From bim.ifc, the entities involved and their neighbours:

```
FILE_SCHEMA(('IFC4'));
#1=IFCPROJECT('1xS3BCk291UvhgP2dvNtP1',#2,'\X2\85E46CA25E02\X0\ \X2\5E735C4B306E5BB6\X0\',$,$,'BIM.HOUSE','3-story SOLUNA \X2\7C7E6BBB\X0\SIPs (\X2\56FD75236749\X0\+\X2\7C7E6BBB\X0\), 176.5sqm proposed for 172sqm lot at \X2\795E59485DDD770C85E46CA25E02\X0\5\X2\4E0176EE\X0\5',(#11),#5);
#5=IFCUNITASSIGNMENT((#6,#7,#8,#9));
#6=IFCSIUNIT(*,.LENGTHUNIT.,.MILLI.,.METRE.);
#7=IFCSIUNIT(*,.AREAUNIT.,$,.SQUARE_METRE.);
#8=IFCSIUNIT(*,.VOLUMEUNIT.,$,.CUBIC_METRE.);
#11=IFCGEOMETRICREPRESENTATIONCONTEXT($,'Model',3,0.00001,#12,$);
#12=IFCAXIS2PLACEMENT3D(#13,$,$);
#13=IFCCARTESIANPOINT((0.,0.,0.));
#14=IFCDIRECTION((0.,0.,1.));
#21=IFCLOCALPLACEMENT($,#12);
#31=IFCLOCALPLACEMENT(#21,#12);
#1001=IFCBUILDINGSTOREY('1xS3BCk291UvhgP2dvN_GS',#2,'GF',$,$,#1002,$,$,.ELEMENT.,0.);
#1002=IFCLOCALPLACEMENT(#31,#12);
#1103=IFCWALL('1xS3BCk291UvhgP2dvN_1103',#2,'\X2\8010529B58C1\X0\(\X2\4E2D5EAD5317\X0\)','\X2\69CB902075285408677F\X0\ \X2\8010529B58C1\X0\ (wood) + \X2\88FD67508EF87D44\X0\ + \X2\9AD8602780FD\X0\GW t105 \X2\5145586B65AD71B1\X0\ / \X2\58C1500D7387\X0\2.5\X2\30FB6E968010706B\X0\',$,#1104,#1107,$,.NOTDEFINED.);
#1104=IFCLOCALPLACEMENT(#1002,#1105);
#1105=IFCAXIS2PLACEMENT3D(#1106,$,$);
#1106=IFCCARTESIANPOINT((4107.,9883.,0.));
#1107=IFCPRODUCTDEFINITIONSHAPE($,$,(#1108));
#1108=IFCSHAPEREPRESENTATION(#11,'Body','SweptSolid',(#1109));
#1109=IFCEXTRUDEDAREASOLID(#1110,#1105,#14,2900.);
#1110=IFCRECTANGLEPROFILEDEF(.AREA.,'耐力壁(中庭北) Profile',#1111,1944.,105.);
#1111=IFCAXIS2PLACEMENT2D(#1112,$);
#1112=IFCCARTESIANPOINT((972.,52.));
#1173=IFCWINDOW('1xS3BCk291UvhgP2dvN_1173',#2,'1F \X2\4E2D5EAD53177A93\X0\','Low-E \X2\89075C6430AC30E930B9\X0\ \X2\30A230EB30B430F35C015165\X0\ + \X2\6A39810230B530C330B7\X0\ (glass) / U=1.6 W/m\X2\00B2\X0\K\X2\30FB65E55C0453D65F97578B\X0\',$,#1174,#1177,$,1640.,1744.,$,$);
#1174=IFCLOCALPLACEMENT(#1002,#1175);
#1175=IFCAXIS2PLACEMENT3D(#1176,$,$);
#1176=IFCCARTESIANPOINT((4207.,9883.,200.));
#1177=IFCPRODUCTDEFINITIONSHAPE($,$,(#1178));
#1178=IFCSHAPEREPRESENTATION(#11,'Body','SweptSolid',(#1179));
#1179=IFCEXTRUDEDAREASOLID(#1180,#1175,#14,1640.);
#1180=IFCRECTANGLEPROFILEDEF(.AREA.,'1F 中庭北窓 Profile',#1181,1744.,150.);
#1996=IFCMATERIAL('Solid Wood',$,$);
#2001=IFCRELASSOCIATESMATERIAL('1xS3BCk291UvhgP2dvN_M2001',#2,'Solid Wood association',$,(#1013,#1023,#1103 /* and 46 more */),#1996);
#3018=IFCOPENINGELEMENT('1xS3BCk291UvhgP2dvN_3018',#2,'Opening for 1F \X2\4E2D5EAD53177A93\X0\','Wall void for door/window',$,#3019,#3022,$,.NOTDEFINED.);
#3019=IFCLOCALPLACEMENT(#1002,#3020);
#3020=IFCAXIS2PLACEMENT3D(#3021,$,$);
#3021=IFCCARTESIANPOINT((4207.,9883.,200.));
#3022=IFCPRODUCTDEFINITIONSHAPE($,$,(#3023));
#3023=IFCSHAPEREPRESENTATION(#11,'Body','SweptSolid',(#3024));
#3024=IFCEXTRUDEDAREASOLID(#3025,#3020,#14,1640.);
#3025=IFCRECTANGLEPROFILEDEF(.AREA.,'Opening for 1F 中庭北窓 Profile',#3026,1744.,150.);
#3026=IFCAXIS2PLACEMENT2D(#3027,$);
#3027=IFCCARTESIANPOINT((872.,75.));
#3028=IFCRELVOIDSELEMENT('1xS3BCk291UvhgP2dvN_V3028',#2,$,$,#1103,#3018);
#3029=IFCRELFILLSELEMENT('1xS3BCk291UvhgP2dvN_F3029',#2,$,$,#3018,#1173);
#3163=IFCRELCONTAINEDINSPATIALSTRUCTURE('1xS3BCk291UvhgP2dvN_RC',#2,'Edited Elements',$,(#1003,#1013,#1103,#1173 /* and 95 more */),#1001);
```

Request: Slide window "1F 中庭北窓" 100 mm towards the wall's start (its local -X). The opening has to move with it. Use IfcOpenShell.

```python
import ifcopenshell
import ifcopenshell.api.geometry
import ifcopenshell.util.placement
import ifcopenshell.util.unit

model = ifcopenshell.open("bim.ifc")
unit_scale = ifcopenshell.util.unit.calculate_unit_scale(model)

window = model.by_id(1173)
opening = window.FillsVoids[0].RelatingOpeningElement
wall = opening.VoidsElements[0].RelatingBuildingElement

wall_matrix = ifcopenshell.util.placement.get_local_placement(wall.ObjectPlacement)
shift = wall_matrix[:3, 0] * -0.1 / unit_scale
before = ifcopenshell.util.placement.get_local_placement(window.ObjectPlacement)[:3, 3].copy()

# The window is not placed relative to its opening, so move both.
for product in (opening, window):
    matrix = ifcopenshell.util.placement.get_local_placement(product.ObjectPlacement)
    matrix[:3, 3] += shift
    ifcopenshell.api.geometry.edit_object_placement(model, product=product, matrix=matrix, is_si=False)

after = ifcopenshell.util.placement.get_local_placement(window.ObjectPlacement)[:3, 3]
print("window moved by", (after - before).round(3) + 0.0)

model.write("bim_v2.ifc")
```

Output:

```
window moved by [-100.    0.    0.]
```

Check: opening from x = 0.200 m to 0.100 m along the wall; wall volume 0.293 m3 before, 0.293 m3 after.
